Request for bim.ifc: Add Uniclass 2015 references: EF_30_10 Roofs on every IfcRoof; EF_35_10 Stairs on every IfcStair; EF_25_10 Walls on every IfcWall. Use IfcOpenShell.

First a look at what the model holds.

```python
import ifcopenshell

model = ifcopenshell.open("bim.ifc")
print(model.schema)
print("classifications:", [c.Name for c in model.by_type("IfcClassification")])
for ifc_class in ("IfcDoor", "IfcRoof", "IfcStair", "IfcWall", "IfcWindow"):
    print(ifc_class, len(model.by_type(ifc_class)))
```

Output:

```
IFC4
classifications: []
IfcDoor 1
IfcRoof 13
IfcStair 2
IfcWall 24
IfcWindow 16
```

```python
import ifcopenshell
import ifcopenshell.api.classification

model = ifcopenshell.open("bim.ifc")

system = ifcopenshell.api.classification.add_classification(model, classification="Uniclass 2015")

codes = {
    "IfcRoof": ("EF_30_10", "Roofs"),
    "IfcStair": ("EF_35_10", "Stairs"),
    "IfcWall": ("EF_25_10", "Walls"),
}
for ifc_class, (code, name) in codes.items():
    products = model.by_type(ifc_class)
    ifcopenshell.api.classification.add_reference(
        model, products=products, classification=system, identification=code, name=name
    )
    print(code, len(products))

model.write("bim_updated.ifc")
```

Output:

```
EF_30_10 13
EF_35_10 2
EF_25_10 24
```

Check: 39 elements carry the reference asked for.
